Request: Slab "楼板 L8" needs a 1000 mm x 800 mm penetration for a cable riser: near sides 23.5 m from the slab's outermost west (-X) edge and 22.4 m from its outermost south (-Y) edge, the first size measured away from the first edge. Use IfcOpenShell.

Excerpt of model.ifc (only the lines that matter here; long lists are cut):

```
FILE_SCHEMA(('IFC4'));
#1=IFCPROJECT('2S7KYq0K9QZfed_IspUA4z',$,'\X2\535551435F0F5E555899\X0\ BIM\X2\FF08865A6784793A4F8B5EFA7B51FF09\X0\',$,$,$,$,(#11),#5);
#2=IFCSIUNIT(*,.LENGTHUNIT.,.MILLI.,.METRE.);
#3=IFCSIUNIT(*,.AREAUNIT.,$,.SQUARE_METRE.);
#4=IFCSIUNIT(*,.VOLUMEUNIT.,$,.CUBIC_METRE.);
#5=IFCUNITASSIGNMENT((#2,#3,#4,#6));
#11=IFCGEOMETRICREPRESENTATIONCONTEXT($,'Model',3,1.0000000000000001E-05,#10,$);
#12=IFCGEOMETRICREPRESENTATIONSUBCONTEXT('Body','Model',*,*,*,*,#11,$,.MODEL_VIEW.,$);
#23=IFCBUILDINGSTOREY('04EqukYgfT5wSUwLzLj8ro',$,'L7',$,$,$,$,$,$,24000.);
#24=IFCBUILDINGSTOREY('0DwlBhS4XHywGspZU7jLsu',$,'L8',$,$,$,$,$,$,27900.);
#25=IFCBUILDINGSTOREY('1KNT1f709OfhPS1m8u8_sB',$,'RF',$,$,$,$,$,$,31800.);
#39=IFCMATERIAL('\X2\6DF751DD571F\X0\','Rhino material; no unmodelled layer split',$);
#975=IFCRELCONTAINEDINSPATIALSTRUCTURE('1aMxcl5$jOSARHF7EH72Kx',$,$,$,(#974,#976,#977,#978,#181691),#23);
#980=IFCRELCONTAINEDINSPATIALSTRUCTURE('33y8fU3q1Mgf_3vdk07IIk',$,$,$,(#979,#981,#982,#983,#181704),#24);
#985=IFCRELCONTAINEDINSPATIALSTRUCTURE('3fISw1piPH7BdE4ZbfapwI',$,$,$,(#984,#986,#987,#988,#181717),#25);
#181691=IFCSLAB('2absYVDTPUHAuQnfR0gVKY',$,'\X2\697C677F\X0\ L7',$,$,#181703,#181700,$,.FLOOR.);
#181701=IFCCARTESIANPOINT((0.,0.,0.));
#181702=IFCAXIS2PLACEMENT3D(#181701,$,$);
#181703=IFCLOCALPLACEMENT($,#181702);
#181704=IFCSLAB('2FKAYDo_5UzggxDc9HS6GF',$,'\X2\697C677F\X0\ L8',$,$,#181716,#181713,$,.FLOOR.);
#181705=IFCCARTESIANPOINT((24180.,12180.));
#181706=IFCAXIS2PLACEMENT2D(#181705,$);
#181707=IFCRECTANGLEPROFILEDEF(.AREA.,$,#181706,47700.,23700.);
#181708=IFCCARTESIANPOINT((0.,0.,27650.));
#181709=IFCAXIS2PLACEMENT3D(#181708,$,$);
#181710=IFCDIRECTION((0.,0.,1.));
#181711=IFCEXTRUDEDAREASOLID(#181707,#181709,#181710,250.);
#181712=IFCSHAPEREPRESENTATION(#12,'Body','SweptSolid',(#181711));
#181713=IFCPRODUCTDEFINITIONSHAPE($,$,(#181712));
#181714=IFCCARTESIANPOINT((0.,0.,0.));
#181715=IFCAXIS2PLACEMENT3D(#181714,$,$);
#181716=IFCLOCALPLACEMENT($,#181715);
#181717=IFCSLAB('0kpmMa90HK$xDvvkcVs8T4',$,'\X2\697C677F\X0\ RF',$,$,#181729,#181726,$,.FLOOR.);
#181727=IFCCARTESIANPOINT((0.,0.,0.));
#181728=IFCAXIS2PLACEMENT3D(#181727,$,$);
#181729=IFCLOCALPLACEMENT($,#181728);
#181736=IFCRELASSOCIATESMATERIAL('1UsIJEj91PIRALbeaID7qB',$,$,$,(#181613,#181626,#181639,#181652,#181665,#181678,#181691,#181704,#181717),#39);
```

```python
import numpy as np
import ifcopenshell
import ifcopenshell.api.feature
import ifcopenshell.api.geometry
import ifcopenshell.api.root
import ifcopenshell.geom
import ifcopenshell.util.placement
import ifcopenshell.util.representation
import ifcopenshell.util.shape
import ifcopenshell.util.unit

model = ifcopenshell.open("model.ifc")
unit_scale = ifcopenshell.util.unit.calculate_unit_scale(model)
settings = ifcopenshell.geom.settings()


def volume(element):
    """Net volume in cubic metres, openings subtracted."""
    shape = ifcopenshell.geom.create_shape(settings, element)
    return ifcopenshell.util.shape.get_volume(shape.geometry)


slab = model.by_guid("2FKAYDo_5UzggxDc9HS6GF")
before = volume(slab)

# Extent in the slab's own axes, in metres. The edges named are its -X and -Y sides.
slab_shape = ifcopenshell.geom.create_shape(settings, slab)
vertices = ifcopenshell.util.shape.get_vertices(slab_shape.geometry)
x_min, y_min, bottom = vertices.min(axis=0)
top = vertices[:, 2].max()

opening = ifcopenshell.api.root.create_entity(model, ifc_class="IfcOpeningElement", name="Cable riser opening", predefined_type="OPENING")
context = ifcopenshell.util.representation.get_context(model, "Model", "Body", "MODEL_VIEW")
width, depth = 1, 0.8
outline = [(0.0, 0.0), (width, 0.0), (width, depth), (0.0, depth), (0.0, 0.0)]
# Overshoot both faces by 50 mm so the cut is clean.
shape = ifcopenshell.api.geometry.add_slab_representation(
    model, context=context, depth=top - bottom + 0.1, polyline=outline
)
ifcopenshell.api.geometry.assign_representation(model, product=opening, representation=shape)

matrix = ifcopenshell.util.placement.get_local_placement(slab.ObjectPlacement)
matrix[:, 3] = matrix @ np.append(np.array([x_min + 23.5, y_min + 22.4, bottom - 0.05]) / unit_scale, 1.0)
ifcopenshell.api.geometry.edit_object_placement(model, product=opening, matrix=matrix, is_si=False)
ifcopenshell.api.feature.add_feature(model, feature=opening, element=slab)

after = volume(slab)

print(f"slab volume {before:.3f} -> {after:.3f} m3")

model.write("model_v2.ifc")
```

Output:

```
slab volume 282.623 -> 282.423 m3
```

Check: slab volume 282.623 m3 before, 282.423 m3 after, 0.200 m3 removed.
